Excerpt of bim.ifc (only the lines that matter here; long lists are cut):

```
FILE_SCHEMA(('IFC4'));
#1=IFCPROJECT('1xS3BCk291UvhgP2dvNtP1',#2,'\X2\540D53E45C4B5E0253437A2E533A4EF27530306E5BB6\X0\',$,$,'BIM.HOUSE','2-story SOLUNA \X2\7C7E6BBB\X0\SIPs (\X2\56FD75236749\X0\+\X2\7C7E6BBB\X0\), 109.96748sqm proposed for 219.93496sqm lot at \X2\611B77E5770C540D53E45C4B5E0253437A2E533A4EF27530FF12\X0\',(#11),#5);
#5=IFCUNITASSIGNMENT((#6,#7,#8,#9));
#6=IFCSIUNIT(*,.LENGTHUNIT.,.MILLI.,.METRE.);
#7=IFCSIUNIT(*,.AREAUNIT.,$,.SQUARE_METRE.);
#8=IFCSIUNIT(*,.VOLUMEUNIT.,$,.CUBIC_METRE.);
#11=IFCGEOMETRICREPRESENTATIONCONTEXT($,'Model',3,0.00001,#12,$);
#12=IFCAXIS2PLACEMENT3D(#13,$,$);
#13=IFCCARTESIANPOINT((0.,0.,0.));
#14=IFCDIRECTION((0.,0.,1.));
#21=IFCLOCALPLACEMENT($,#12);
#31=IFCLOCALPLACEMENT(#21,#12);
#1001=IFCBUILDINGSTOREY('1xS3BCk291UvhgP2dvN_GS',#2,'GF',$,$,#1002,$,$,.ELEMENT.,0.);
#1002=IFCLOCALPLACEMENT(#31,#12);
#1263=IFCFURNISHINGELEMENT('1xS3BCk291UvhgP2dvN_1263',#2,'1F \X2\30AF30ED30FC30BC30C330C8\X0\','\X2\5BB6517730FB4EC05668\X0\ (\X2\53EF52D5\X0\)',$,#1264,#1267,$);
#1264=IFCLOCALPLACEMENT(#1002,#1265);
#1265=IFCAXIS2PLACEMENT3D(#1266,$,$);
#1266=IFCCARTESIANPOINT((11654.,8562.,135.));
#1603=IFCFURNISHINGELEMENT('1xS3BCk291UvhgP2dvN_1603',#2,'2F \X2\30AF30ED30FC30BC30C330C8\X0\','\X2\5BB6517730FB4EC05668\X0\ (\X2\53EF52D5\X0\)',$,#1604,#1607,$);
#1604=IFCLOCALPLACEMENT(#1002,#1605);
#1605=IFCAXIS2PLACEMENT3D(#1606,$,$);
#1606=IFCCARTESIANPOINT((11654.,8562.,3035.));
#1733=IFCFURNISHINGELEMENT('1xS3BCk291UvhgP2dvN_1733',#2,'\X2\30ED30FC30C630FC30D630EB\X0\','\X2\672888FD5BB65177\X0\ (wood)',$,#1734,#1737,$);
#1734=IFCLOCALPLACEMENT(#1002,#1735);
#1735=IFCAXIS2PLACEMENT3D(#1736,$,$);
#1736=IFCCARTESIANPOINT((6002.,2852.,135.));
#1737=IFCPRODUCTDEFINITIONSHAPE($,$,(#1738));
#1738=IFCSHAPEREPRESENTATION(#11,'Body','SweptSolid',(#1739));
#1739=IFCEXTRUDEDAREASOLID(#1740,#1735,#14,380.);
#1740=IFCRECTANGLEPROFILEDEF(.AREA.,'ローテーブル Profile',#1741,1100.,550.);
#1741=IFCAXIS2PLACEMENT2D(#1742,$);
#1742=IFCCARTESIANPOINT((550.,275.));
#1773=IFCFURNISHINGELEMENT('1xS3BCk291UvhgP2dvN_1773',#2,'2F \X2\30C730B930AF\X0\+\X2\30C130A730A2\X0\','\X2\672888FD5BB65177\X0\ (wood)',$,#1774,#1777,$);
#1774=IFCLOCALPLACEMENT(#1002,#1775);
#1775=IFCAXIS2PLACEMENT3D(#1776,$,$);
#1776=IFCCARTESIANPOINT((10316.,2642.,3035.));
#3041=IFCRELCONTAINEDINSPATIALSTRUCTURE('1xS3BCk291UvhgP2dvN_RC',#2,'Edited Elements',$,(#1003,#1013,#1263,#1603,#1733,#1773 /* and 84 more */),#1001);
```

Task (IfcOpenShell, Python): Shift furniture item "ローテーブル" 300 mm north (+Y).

```python
import ifcopenshell
import ifcopenshell.api.geometry
import ifcopenshell.util.placement

model = ifcopenshell.open("bim.ifc")

item = model.by_id(1733)
matrix = ifcopenshell.util.placement.get_local_placement(item.ObjectPlacement)
matrix[1, 3] += 300.0
ifcopenshell.api.geometry.edit_object_placement(model, product=item, matrix=matrix, is_si=False)

print(ifcopenshell.util.placement.get_local_placement(item.ObjectPlacement).round(3) + 0.0)

model.write("bim_edited.ifc")
```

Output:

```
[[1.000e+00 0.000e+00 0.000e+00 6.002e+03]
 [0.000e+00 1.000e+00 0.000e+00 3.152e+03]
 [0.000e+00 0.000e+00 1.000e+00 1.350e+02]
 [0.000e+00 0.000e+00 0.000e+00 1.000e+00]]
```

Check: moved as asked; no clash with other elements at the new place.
